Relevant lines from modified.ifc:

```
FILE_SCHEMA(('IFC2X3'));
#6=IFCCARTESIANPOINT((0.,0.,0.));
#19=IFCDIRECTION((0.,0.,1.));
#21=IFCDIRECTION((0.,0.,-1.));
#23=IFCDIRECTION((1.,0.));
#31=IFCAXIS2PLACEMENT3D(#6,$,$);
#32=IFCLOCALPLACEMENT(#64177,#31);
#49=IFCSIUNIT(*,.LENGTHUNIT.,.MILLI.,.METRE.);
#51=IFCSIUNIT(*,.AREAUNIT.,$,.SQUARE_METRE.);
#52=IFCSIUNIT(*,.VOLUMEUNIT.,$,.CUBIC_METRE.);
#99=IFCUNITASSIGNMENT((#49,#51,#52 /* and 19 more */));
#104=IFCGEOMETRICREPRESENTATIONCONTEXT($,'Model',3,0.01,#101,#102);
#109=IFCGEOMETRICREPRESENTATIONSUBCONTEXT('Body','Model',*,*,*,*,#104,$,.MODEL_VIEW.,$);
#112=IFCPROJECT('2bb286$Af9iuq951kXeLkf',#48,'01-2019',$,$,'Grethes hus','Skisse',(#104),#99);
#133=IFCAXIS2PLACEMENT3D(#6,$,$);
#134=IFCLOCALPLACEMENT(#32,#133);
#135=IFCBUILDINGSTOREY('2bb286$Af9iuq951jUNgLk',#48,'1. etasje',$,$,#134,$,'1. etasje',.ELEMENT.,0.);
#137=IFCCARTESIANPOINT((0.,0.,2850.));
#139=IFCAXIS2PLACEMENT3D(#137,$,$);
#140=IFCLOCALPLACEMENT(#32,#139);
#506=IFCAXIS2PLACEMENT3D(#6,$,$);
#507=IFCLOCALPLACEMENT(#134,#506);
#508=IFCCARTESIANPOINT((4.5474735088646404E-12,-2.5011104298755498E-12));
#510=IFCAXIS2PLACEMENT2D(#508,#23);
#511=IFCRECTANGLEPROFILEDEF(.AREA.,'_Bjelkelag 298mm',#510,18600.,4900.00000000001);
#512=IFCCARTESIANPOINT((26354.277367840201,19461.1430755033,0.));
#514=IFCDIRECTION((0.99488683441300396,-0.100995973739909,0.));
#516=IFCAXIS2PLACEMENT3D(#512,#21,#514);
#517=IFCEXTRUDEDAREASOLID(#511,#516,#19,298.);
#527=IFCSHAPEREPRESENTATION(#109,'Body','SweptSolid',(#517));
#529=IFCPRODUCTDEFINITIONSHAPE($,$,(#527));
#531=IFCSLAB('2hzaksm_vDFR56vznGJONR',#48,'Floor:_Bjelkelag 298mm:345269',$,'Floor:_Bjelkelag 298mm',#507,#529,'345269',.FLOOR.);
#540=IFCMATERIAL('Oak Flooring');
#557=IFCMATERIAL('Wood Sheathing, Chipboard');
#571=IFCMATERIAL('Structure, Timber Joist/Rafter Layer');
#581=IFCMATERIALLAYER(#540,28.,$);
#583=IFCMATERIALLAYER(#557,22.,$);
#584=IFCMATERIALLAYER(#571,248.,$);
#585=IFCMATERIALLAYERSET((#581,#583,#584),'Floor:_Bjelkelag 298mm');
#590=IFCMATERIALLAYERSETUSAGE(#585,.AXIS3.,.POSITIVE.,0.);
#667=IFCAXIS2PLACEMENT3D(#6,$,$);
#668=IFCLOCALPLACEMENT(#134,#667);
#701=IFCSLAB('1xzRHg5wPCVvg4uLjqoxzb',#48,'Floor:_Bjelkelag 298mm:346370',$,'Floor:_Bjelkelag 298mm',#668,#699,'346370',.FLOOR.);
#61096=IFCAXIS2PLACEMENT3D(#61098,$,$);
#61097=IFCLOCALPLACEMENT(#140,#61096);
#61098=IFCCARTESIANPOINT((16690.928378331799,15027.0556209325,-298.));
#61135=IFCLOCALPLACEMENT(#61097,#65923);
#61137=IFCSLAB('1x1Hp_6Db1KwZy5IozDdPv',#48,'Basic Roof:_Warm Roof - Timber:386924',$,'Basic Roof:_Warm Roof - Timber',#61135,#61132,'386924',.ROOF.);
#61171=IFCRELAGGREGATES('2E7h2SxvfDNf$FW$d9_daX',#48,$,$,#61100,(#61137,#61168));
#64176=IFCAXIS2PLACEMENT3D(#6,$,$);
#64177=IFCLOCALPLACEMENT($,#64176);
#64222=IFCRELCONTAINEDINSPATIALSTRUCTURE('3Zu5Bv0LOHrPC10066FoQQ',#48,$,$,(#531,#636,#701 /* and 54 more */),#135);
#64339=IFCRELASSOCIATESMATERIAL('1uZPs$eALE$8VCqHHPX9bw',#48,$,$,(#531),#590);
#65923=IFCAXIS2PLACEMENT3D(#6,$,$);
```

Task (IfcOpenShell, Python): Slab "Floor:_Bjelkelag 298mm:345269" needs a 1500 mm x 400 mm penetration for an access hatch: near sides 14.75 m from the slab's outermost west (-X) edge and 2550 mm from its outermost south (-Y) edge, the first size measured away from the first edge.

```python
import numpy as np
import ifcopenshell
import ifcopenshell.api.feature
import ifcopenshell.api.geometry
import ifcopenshell.api.root
import ifcopenshell.geom
import ifcopenshell.util.placement
import ifcopenshell.util.representation
import ifcopenshell.util.shape
import ifcopenshell.util.unit

model = ifcopenshell.open("modified.ifc")
unit_scale = ifcopenshell.util.unit.calculate_unit_scale(model)
settings = ifcopenshell.geom.settings()


def volume(element):
    """Net volume in cubic metres, openings subtracted."""
    shape = ifcopenshell.geom.create_shape(settings, element)
    return ifcopenshell.util.shape.get_volume(shape.geometry)


slab = model.by_guid("2hzaksm_vDFR56vznGJONR")
before = volume(slab)

# Extent in the slab's own axes, in metres. The edges named are its -X and -Y sides.
slab_shape = ifcopenshell.geom.create_shape(settings, slab)
vertices = ifcopenshell.util.shape.get_vertices(slab_shape.geometry)
x_min, y_min, bottom = vertices.min(axis=0)
top = vertices[:, 2].max()

opening = ifcopenshell.api.root.create_entity(model, ifc_class="IfcOpeningElement", name="Access hatch opening")
context = ifcopenshell.util.representation.get_context(model, "Model", "Body", "MODEL_VIEW")
width, depth = 1.5, 0.4
outline = [(0.0, 0.0), (width, 0.0), (width, depth), (0.0, depth), (0.0, 0.0)]
# Overshoot both faces by 50 mm so the cut is clean.
shape = ifcopenshell.api.geometry.add_slab_representation(
    model, context=context, depth=top - bottom + 0.1, polyline=outline
)
ifcopenshell.api.geometry.assign_representation(model, product=opening, representation=shape)

matrix = ifcopenshell.util.placement.get_local_placement(slab.ObjectPlacement)
matrix[:, 3] = matrix @ np.append(np.array([x_min + 14.75, y_min + 2.55, bottom - 0.05]) / unit_scale, 1.0)
ifcopenshell.api.geometry.edit_object_placement(model, product=opening, matrix=matrix, is_si=False)
ifcopenshell.api.feature.add_feature(model, feature=opening, element=slab)

after = volume(slab)

print(f"slab volume {before:.3f} -> {after:.3f} m3")

model.write("modified_updated.ifc")
```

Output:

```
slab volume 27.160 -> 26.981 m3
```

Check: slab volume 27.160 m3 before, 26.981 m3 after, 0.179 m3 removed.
